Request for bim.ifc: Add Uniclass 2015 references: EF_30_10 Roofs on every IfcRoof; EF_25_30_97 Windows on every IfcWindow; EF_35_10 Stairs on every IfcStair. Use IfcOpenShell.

First a look at what the model holds.

```python
import ifcopenshell

model = ifcopenshell.open("bim.ifc")
print(model.schema)
print("classifications:", [c.Name for c in model.by_type("IfcClassification")])
for ifc_class in ("IfcDoor", "IfcRoof", "IfcStair", "IfcWall", "IfcWindow"):
    print(ifc_class, len(model.by_type(ifc_class)))
```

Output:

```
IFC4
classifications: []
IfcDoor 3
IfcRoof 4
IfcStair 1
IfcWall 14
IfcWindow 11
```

```python
import ifcopenshell
import ifcopenshell.api.classification

model = ifcopenshell.open("bim.ifc")

system = ifcopenshell.api.classification.add_classification(model, classification="Uniclass 2015")

codes = {
    "IfcRoof": ("EF_30_10", "Roofs"),
    "IfcWindow": ("EF_25_30_97", "Windows"),
    "IfcStair": ("EF_35_10", "Stairs"),
}
for ifc_class, (code, name) in codes.items():
    products = model.by_type(ifc_class)
    ifcopenshell.api.classification.add_reference(
        model, products=products, classification=system, identification=code, name=name
    )
    print(code, len(products))

model.write("bim-out.ifc")
```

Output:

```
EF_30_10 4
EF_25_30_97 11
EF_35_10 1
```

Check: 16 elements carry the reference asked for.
